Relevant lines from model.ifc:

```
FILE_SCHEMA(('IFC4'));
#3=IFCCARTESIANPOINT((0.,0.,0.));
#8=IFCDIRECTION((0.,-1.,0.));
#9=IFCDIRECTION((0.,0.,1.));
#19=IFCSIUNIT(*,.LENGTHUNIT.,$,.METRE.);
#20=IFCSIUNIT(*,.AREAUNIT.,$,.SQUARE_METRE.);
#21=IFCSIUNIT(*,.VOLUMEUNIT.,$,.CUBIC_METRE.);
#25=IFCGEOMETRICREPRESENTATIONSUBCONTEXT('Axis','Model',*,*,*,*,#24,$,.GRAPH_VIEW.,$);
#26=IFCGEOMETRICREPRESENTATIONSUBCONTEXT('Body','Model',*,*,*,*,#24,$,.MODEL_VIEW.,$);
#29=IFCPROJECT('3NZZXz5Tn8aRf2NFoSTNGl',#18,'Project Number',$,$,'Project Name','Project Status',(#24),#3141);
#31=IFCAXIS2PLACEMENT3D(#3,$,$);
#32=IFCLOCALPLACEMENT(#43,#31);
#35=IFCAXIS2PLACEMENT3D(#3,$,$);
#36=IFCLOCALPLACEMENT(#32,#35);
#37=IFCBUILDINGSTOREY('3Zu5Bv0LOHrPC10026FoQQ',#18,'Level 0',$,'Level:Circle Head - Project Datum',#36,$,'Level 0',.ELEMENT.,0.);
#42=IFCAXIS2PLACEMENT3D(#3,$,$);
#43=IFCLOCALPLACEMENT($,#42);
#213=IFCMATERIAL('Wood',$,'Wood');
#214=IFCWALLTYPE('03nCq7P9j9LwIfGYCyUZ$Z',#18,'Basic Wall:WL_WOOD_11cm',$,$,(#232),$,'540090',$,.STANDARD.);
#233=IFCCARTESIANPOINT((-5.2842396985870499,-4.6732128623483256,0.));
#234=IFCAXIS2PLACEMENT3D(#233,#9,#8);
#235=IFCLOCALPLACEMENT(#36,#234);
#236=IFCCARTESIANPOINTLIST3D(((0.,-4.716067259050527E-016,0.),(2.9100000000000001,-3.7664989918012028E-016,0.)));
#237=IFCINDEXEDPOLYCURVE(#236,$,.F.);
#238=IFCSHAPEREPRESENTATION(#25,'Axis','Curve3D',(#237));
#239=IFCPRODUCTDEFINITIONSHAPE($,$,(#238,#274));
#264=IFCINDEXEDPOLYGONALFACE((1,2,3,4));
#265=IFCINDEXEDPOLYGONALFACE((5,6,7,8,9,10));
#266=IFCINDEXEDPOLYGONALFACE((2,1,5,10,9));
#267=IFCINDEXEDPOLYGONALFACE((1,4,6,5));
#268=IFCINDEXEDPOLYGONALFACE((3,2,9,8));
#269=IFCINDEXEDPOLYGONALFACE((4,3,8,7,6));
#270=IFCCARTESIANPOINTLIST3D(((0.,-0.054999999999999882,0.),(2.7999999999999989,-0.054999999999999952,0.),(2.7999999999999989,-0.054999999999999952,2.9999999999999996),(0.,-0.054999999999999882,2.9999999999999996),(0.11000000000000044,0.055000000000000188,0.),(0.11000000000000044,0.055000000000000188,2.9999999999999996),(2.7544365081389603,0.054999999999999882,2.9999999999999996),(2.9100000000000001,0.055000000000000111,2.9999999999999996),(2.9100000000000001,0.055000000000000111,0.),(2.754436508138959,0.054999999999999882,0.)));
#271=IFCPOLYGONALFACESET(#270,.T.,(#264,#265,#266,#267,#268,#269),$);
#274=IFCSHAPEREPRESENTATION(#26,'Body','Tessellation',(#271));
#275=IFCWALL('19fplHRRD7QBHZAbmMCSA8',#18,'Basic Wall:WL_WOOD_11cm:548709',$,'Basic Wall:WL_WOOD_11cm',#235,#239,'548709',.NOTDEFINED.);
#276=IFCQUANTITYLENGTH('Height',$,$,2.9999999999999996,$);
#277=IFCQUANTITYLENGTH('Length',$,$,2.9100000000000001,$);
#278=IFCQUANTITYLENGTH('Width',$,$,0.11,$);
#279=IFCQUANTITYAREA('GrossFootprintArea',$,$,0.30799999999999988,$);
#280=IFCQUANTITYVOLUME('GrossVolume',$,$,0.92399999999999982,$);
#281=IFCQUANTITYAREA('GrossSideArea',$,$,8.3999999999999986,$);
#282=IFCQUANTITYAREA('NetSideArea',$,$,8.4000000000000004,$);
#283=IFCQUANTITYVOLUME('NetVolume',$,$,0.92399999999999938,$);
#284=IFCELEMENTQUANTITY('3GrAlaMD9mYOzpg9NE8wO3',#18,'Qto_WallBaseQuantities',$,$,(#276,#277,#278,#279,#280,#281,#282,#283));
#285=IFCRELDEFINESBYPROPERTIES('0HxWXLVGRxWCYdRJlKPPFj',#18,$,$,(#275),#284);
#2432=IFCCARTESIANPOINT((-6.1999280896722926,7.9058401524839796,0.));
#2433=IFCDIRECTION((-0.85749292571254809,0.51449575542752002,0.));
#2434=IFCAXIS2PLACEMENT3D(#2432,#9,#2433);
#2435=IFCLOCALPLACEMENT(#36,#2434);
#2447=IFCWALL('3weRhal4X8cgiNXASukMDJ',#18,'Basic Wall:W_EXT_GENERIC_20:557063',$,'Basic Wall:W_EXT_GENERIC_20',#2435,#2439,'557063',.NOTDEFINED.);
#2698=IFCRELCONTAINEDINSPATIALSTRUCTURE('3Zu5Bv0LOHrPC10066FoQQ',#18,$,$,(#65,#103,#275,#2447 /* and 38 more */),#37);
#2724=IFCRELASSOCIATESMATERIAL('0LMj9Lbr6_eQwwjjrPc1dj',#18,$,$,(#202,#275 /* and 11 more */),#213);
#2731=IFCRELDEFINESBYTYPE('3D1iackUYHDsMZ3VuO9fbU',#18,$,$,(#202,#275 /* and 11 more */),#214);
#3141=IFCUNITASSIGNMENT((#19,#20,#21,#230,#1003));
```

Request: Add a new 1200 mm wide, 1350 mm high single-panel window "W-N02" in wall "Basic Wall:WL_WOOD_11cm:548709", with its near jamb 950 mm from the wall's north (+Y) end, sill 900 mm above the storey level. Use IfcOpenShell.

```python
import numpy as np
import ifcopenshell
import ifcopenshell.api.feature
import ifcopenshell.api.geometry
import ifcopenshell.api.pset
import ifcopenshell.api.root
import ifcopenshell.api.spatial
import ifcopenshell.geom
import ifcopenshell.util.element
import ifcopenshell.util.placement
import ifcopenshell.util.representation
import ifcopenshell.util.shape
import ifcopenshell.util.unit

model = ifcopenshell.open("model.ifc")
unit_scale = ifcopenshell.util.unit.calculate_unit_scale(model)
area_scale = ifcopenshell.util.unit.calculate_unit_scale(model, "AREAUNIT")
volume_scale = ifcopenshell.util.unit.calculate_unit_scale(model, "VOLUMEUNIT")
settings = ifcopenshell.geom.settings()


def volume(element):
    """Net volume in cubic metres, openings subtracted."""
    shape = ifcopenshell.geom.create_shape(settings, element)
    return ifcopenshell.util.shape.get_volume(shape.geometry)


wall = model.by_guid("19fplHRRD7QBHZAbmMCSA8")
storey = ifcopenshell.util.element.get_container(wall, ifc_class="IfcBuildingStorey")
context = ifcopenshell.util.representation.get_context(model, "Model", "Body", "MODEL_VIEW")
before = volume(wall)

width, height, from_end, sill = 1.2, 1.35, 0.95, 0.9  # metres

# The wall runs along its own X axis, and the end named is its -X end.
wall_shape = ifcopenshell.geom.create_shape(settings, wall)
x, y, z = ifcopenshell.util.shape.get_vertices(wall_shape.geometry).T
start = x.min() + from_end
face, thickness = float(y.min()), float(y.max() - y.min())
wall_matrix = ifcopenshell.util.placement.get_local_placement(wall.ObjectPlacement)
level = ifcopenshell.util.placement.get_local_placement(storey.ObjectPlacement)[2, 3]


def in_wall(x, y):
    """Placement at x, y metres in the wall's axes, at sill height."""
    matrix = wall_matrix.copy()
    matrix[:, 3] = wall_matrix @ np.array([x / unit_scale, y / unit_scale, 0.0, 1.0])
    matrix[2, 3] = level + sill / unit_scale
    return matrix


# Opening: a box that overshoots both wall faces by 50 mm.
opening = ifcopenshell.api.root.create_entity(model, ifc_class="IfcOpeningElement", predefined_type="OPENING")
box = ifcopenshell.api.geometry.add_wall_representation(
    model, context=context, length=width, height=height, thickness=thickness + 0.1
)
ifcopenshell.api.geometry.assign_representation(model, product=opening, representation=box)
ifcopenshell.api.geometry.edit_object_placement(model, product=opening, matrix=in_wall(start, face - 0.05), is_si=False)
ifcopenshell.api.feature.add_feature(model, feature=opening, element=wall)

window = ifcopenshell.api.root.create_entity(model, ifc_class="IfcWindow", name="W-N02", predefined_type="WINDOW")
window.OverallWidth, window.OverallHeight = width / unit_scale, height / unit_scale
window.PartitioningType = "SINGLE_PANEL"
body = ifcopenshell.api.geometry.add_window_representation(
    model,
    context=context,
    overall_width=window.OverallWidth,
    overall_height=window.OverallHeight,
    partition_type="SINGLE_PANEL",
)
ifcopenshell.api.geometry.assign_representation(model, product=window, representation=body)
ifcopenshell.api.spatial.assign_container(model, products=[window], relating_structure=storey)
ifcopenshell.api.feature.add_filling(model, opening=opening, element=window)

# Centre the window in the wall's thickness.
ifcopenshell.api.geometry.edit_object_placement(model, product=window, matrix=in_wall(start, face), is_si=False)
window_shape = ifcopenshell.geom.create_shape(settings, window)
depth = ifcopenshell.util.shape.get_vertices(window_shape.geometry)[:, 1]
offset = face + thickness / 2 - (depth.min() + depth.max()) / 2
ifcopenshell.api.geometry.edit_object_placement(model, product=window, matrix=in_wall(start, offset), is_si=False)

after = volume(wall)

# Update the wall's stored quantities.
qto = model.by_id(ifcopenshell.util.element.get_pset(wall, "Qto_WallBaseQuantities", should_inherit=False)["id"])
ifcopenshell.api.pset.edit_qto(model, qto=qto, properties={
    "NetSideArea": after / thickness / area_scale,
    "NetVolume": after / volume_scale,
})

print(f"wall volume {before:.3f} -> {after:.3f} m3")

model.write("model-out.ifc")
```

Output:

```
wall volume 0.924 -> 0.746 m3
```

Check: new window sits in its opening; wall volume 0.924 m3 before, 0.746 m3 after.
